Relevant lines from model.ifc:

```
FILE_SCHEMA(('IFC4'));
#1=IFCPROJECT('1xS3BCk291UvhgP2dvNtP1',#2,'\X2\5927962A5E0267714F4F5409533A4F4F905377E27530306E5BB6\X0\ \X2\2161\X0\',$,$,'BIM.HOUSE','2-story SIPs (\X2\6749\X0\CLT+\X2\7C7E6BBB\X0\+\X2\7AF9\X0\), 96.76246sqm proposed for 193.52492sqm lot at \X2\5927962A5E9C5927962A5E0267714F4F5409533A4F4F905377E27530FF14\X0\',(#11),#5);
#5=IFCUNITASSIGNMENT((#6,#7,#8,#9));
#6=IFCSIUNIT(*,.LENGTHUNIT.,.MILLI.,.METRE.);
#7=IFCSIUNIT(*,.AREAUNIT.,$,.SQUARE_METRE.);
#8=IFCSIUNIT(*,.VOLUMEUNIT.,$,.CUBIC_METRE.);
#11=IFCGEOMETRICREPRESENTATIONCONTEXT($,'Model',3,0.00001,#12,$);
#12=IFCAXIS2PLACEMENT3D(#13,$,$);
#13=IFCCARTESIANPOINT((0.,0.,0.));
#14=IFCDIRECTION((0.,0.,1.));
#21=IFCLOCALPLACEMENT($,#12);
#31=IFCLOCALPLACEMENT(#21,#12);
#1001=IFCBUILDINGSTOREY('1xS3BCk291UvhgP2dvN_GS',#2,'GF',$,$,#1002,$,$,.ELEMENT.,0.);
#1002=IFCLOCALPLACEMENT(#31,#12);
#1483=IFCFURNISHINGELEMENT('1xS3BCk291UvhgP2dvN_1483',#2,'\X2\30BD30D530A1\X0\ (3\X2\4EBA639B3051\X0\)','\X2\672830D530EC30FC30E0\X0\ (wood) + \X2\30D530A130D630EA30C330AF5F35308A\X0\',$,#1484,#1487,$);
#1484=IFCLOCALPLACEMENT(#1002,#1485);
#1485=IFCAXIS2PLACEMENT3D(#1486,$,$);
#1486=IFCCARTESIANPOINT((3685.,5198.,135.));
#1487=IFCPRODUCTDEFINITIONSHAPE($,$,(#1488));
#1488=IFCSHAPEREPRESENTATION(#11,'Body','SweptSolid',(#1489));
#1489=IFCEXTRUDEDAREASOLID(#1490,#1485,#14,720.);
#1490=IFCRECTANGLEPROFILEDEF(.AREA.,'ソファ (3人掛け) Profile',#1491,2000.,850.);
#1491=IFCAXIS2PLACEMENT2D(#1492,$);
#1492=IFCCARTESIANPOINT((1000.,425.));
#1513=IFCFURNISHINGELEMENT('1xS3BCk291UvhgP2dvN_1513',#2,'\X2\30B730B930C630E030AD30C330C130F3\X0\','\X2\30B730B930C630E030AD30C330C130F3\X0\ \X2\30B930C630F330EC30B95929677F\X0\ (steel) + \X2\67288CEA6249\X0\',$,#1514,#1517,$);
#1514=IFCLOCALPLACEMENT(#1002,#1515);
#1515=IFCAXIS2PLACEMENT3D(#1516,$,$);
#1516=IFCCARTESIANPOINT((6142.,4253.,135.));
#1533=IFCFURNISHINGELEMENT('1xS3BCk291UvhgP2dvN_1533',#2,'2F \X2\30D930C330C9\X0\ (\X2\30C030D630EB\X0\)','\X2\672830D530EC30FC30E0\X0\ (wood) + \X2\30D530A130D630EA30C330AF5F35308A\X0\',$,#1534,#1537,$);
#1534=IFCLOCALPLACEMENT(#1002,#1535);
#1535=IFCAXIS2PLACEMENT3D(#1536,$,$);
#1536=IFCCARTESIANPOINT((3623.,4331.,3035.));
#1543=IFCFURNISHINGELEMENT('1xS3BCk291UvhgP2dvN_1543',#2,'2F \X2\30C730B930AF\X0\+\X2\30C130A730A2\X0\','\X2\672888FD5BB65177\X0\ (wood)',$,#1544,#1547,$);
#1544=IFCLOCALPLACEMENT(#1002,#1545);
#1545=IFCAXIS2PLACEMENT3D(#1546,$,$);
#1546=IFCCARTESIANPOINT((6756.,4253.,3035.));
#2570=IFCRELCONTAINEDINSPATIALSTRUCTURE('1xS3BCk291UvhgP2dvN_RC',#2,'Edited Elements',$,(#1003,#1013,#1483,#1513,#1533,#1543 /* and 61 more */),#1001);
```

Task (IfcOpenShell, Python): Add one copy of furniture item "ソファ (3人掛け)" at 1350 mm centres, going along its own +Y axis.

```python
import ifcopenshell
import ifcopenshell.api.geometry
import ifcopenshell.api.root
import ifcopenshell.util.element
import ifcopenshell.util.placement
import ifcopenshell.util.unit

model = ifcopenshell.open("model.ifc")
unit_scale = ifcopenshell.util.unit.calculate_unit_scale(model)


def reuse_history(source, copy):
    """copy_class also copies each property set's owner history, people and application; keep the originals."""
    for rel in copy.IsDefinedBy:
        if rel.is_a("IfcRelDefinesByProperties") and (history := rel.RelatingPropertyDefinition.OwnerHistory):
            rel.RelatingPropertyDefinition.OwnerHistory = source.OwnerHistory
            ifcopenshell.util.element.remove_deep2(model, history)


source = model.by_guid("1xS3BCk291UvhgP2dvN_1483")
base = ifcopenshell.util.placement.get_local_placement(source.ObjectPlacement)
step = base[:3, 1] * 1.35 / unit_scale

for i in range(1, 2):
    copy = ifcopenshell.api.root.copy_class(model, product=source)
    copy.Representation = ifcopenshell.util.element.copy_deep(
        model, source.Representation, exclude=["IfcGeometricRepresentationContext", "IfcRepresentationMap"]
    )
    reuse_history(source, copy)
    matrix = base.copy()
    matrix[:3, 3] += i * step
    print("added at", matrix[:3, 3].round(3) + 0.0)
    ifcopenshell.api.geometry.edit_object_placement(model, product=copy, matrix=matrix, is_si=False)

model.write("model_updated.ifc")
```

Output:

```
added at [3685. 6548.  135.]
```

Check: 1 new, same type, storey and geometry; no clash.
